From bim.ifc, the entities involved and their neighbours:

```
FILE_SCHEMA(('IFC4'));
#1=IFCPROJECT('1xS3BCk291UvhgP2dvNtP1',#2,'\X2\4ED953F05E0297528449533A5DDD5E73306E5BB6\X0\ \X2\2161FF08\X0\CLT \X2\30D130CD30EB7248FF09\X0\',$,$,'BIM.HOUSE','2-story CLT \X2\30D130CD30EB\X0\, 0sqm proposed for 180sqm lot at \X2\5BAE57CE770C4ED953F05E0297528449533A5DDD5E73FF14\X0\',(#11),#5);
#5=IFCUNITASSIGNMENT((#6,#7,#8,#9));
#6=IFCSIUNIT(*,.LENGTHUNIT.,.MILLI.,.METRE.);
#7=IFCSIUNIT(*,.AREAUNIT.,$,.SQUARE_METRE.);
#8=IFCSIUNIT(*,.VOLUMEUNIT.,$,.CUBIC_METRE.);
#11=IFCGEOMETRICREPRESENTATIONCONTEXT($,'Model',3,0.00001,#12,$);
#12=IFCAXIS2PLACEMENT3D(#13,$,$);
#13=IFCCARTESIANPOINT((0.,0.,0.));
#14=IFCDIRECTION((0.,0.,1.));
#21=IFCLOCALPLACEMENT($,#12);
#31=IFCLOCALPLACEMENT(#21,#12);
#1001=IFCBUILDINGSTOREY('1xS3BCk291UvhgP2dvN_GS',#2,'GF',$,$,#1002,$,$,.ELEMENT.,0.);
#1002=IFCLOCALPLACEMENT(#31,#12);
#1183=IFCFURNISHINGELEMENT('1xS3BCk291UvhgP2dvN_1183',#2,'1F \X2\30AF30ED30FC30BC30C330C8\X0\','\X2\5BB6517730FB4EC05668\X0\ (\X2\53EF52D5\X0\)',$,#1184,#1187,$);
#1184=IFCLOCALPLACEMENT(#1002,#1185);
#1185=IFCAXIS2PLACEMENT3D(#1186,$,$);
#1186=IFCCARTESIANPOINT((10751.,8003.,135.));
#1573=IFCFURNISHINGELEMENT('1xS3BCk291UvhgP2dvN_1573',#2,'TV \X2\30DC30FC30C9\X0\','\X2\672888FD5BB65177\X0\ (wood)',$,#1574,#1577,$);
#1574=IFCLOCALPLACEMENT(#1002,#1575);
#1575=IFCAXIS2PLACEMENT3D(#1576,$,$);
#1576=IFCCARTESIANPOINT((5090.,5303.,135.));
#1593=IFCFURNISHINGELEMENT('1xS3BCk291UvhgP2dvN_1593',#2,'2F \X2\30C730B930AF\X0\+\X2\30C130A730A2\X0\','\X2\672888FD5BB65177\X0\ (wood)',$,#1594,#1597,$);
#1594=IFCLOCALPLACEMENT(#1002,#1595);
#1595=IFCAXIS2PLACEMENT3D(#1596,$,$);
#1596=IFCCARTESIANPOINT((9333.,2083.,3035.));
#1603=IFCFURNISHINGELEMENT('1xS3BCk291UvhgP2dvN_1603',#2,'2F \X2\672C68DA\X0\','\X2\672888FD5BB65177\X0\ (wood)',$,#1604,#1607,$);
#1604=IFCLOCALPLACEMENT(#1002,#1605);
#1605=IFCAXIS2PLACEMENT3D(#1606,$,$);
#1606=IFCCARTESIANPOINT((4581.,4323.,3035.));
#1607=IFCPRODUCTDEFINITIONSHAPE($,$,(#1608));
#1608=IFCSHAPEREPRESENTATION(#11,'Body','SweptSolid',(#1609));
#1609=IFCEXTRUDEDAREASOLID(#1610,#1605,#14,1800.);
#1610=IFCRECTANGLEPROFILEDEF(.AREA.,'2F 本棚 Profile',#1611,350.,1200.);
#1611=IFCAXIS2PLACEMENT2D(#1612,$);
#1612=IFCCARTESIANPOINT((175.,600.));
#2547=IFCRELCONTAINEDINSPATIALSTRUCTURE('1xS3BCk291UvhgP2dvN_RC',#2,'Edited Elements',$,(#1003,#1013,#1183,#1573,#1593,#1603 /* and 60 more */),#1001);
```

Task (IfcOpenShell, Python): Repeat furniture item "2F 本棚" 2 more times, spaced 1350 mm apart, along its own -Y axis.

```python
import ifcopenshell
import ifcopenshell.api.geometry
import ifcopenshell.api.root
import ifcopenshell.util.element
import ifcopenshell.util.placement

model = ifcopenshell.open("bim.ifc")


def reuse_history(source, copy):
    """copy_class also copies each property set's owner history, people and application; keep the originals."""
    for rel in copy.IsDefinedBy:
        if rel.is_a("IfcRelDefinesByProperties") and (history := rel.RelatingPropertyDefinition.OwnerHistory):
            rel.RelatingPropertyDefinition.OwnerHistory = source.OwnerHistory
            ifcopenshell.util.element.remove_deep2(model, history)


source = model.by_guid("1xS3BCk291UvhgP2dvN_1603")
base = ifcopenshell.util.placement.get_local_placement(source.ObjectPlacement)
step = -base[:3, 1] * 1350.0

for i in range(1, 3):
    copy = ifcopenshell.api.root.copy_class(model, product=source)
    copy.Representation = ifcopenshell.util.element.copy_deep(
        model, source.Representation, exclude=["IfcGeometricRepresentationContext", "IfcRepresentationMap"]
    )
    reuse_history(source, copy)
    matrix = base.copy()
    matrix[:3, 3] += i * step
    print("added at", matrix[:3, 3].round(3) + 0.0)
    ifcopenshell.api.geometry.edit_object_placement(model, product=copy, matrix=matrix, is_si=False)

model.write("bim-out.ifc")
```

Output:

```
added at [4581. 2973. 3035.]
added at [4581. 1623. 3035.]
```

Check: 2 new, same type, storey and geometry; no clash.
